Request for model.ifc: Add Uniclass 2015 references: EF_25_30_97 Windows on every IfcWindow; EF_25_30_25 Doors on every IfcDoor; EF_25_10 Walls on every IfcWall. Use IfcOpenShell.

First a look at what the model holds.

```python
import ifcopenshell

model = ifcopenshell.open("model.ifc")
print(model.schema)
print("classifications:", [c.Name for c in model.by_type("IfcClassification")])
for ifc_class in ("IfcDoor", "IfcRoof", "IfcStair", "IfcWall", "IfcWindow"):
    print(ifc_class, len(model.by_type(ifc_class)))
```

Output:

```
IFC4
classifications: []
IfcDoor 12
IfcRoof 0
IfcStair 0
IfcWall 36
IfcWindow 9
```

```python
import ifcopenshell
import ifcopenshell.api.classification

model = ifcopenshell.open("model.ifc")

system = ifcopenshell.api.classification.add_classification(model, classification="Uniclass 2015")

codes = {
    "IfcWindow": ("EF_25_30_97", "Windows"),
    "IfcDoor": ("EF_25_30_25", "Doors"),
    "IfcWall": ("EF_25_10", "Walls"),
}
for ifc_class, (code, name) in codes.items():
    products = model.by_type(ifc_class)
    ifcopenshell.api.classification.add_reference(
        model, products=products, classification=system, identification=code, name=name
    )
    print(code, len(products))

model.write("model_updated.ifc")
```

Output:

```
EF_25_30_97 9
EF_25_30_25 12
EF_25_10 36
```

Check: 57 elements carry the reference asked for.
